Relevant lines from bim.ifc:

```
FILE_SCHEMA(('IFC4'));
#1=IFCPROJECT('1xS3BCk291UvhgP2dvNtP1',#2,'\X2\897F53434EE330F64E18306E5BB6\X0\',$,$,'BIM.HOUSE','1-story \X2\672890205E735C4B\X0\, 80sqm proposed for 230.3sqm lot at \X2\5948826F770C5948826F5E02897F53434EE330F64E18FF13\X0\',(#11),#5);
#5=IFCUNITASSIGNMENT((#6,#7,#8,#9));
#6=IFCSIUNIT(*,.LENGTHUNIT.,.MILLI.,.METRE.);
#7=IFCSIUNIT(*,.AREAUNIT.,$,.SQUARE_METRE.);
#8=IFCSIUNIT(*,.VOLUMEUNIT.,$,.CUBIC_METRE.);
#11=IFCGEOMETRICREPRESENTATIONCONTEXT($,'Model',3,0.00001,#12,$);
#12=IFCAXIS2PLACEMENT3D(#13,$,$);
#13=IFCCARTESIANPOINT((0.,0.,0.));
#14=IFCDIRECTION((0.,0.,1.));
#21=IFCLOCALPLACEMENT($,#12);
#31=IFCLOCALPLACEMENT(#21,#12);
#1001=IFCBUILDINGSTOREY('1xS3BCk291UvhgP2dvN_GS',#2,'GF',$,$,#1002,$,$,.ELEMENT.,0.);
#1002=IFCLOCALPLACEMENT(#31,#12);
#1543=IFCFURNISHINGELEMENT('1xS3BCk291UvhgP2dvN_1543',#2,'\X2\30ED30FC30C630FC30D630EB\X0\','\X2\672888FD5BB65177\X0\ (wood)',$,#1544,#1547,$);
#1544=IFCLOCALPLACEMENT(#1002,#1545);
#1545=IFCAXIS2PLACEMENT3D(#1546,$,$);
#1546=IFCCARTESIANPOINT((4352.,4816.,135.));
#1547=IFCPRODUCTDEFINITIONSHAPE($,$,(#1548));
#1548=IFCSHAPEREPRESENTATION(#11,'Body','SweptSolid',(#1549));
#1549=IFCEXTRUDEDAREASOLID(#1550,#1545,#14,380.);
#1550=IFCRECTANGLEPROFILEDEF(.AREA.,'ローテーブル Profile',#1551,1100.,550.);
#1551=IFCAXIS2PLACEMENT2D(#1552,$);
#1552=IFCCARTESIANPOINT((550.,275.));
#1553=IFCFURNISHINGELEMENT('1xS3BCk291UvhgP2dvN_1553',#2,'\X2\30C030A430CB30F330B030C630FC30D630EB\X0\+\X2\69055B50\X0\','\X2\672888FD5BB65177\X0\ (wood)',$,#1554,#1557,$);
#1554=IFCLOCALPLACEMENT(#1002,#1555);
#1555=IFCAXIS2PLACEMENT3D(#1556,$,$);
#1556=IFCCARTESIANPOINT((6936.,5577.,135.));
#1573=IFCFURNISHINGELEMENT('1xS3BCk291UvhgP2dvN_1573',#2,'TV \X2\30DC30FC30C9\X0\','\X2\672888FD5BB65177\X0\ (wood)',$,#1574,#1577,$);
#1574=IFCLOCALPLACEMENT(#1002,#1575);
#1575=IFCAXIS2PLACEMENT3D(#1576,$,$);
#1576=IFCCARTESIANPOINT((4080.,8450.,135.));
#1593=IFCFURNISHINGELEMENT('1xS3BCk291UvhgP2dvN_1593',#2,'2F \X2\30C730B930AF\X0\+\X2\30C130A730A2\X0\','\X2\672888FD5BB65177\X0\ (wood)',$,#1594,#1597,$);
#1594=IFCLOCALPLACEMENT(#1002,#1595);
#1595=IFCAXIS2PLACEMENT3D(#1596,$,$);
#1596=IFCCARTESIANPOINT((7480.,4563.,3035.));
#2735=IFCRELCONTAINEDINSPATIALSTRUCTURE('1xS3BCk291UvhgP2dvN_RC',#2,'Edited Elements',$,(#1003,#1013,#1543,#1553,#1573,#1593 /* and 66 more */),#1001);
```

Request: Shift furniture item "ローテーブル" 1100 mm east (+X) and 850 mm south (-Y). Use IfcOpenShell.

```python
import ifcopenshell
import ifcopenshell.api.geometry
import ifcopenshell.util.placement

model = ifcopenshell.open("bim.ifc")

item = model.by_guid("1xS3BCk291UvhgP2dvN_1543")
matrix = ifcopenshell.util.placement.get_local_placement(item.ObjectPlacement)
matrix[0, 3] += 1100.0
matrix[1, 3] -= 850.0
ifcopenshell.api.geometry.edit_object_placement(model, product=item, matrix=matrix, is_si=False)

print(ifcopenshell.util.placement.get_local_placement(item.ObjectPlacement).round(3) + 0.0)

model.write("bim_edited.ifc")
```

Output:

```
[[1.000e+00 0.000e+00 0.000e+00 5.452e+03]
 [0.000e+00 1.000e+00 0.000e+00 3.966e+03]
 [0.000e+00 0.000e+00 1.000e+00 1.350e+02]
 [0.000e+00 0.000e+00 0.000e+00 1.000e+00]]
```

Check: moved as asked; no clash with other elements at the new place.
